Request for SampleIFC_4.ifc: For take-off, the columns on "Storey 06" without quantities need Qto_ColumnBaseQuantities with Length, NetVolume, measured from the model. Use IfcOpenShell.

First a look at what the model holds.

```python
import ifcopenshell
import ifcopenshell.util.element
import ifcopenshell.util.unit

model = ifcopenshell.open("SampleIFC_4.ifc")
print(model.schema)
for unit_type in ("LENGTHUNIT", "AREAUNIT", "VOLUMEUNIT"):
    print(unit_type, ifcopenshell.util.unit.calculate_unit_scale(model, unit_type))
storey = next(s for s in model.by_type("IfcBuildingStorey") if s.Name == "Storey 06")
columns = [e for e in ifcopenshell.util.element.get_decomposition(storey) if e.is_a("IfcColumn")]
for e in sorted(columns, key=lambda e: e.id()):
    print(e.id(), e.is_a(), e.Name, list(ifcopenshell.util.element.get_psets(e, qtos_only=True)), sep=" | ")
```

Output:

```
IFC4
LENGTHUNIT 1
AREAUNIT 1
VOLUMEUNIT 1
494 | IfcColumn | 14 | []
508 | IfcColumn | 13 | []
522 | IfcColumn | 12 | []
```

```python
import ifcopenshell
import ifcopenshell.api.pset
import ifcopenshell.geom
import ifcopenshell.util.element
import ifcopenshell.util.shape
import ifcopenshell.util.unit

model = ifcopenshell.open("SampleIFC_4.ifc")
unit_scale = ifcopenshell.util.unit.calculate_unit_scale(model)
volume_scale = ifcopenshell.util.unit.calculate_unit_scale(model, "VOLUMEUNIT")
settings = ifcopenshell.geom.settings()

storey = next(s for s in model.by_type("IfcBuildingStorey") if s.Name == "Storey 06")
columns = [e for e in ifcopenshell.util.element.get_decomposition(storey) if e.is_a("IfcColumn")]

for e in sorted(columns, key=lambda e: e.id()):
    if ifcopenshell.util.element.get_psets(e, qtos_only=True, should_inherit=False):
        continue
    # Geometry comes back in metres, in the element's own axes.
    shape = ifcopenshell.geom.create_shape(settings, e)
    values = {
        "Length": ifcopenshell.util.shape.get_z(shape.geometry) / unit_scale,
        "NetVolume": ifcopenshell.util.shape.get_volume(shape.geometry) / volume_scale,
    }
    qto = ifcopenshell.api.pset.add_qto(model, product=e, name="Qto_ColumnBaseQuantities")
    ifcopenshell.api.pset.edit_qto(model, qto=qto, properties=values)
    print(e.id(), {k: round(v, 3) for k, v in values.items()})

model.write("SampleIFC_4_v2.ifc")
```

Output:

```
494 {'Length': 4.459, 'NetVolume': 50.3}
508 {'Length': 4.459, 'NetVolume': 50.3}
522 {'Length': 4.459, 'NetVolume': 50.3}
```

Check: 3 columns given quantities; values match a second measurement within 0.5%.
